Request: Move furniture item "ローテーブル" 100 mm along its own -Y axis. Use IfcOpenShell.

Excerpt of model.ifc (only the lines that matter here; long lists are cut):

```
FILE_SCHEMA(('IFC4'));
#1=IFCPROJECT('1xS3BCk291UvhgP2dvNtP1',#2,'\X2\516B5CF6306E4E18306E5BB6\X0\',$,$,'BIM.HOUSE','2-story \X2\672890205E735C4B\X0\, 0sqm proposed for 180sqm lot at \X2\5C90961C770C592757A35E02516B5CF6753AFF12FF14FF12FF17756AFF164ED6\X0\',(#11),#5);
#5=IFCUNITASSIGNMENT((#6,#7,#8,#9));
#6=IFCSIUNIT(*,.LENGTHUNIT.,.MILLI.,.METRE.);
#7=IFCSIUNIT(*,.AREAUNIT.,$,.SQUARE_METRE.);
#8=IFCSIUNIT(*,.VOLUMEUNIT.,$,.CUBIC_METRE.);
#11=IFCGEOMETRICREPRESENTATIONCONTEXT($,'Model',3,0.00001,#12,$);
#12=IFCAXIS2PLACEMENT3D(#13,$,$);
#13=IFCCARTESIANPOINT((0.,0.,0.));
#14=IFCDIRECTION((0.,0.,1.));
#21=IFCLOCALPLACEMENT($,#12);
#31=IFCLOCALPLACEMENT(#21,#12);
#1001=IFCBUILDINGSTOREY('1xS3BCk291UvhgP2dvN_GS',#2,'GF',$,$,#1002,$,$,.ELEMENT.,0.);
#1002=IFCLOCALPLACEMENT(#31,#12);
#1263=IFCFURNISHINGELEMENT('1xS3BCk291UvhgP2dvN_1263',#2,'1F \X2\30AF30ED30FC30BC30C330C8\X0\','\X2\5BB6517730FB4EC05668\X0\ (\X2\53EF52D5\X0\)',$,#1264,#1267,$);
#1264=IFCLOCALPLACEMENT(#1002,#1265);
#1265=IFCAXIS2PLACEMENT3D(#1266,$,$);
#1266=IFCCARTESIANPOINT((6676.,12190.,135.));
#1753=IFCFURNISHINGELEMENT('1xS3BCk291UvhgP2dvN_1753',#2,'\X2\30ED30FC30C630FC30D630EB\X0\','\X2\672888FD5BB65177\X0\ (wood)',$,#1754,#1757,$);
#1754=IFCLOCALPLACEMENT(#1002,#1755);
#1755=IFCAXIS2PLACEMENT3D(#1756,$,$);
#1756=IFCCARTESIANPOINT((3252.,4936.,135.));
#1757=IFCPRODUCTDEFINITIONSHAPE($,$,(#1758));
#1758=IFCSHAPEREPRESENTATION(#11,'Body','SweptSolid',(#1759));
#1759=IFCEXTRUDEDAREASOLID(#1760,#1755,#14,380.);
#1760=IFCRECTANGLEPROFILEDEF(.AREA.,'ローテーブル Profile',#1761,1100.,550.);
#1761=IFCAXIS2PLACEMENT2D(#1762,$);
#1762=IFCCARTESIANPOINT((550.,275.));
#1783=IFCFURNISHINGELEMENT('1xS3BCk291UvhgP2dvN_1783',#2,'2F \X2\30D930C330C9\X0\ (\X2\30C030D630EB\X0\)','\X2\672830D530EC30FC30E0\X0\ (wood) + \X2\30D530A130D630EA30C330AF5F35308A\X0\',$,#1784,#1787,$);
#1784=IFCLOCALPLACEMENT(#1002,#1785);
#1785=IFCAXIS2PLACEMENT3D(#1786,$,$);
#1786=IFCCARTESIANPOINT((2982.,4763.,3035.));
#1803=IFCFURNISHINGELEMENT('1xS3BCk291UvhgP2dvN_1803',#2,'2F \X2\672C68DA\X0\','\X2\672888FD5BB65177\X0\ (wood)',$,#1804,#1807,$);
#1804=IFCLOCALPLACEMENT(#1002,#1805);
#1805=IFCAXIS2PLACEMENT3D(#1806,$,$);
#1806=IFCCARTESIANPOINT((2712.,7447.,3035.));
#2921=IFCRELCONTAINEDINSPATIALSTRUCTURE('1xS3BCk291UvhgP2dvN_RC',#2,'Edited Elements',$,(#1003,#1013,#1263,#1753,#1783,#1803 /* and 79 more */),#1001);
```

```python
import ifcopenshell
import ifcopenshell.api.geometry
import ifcopenshell.util.placement
import ifcopenshell.util.unit

model = ifcopenshell.open("model.ifc")
unit_scale = ifcopenshell.util.unit.calculate_unit_scale(model)

item = model.by_guid("1xS3BCk291UvhgP2dvN_1753")
matrix = ifcopenshell.util.placement.get_local_placement(item.ObjectPlacement)
matrix[:3, 3] -= matrix[:3, 1] * 0.1 / unit_scale
ifcopenshell.api.geometry.edit_object_placement(model, product=item, matrix=matrix, is_si=False)

print(ifcopenshell.util.placement.get_local_placement(item.ObjectPlacement).round(3) + 0.0)

model.write("model_rev.ifc")
```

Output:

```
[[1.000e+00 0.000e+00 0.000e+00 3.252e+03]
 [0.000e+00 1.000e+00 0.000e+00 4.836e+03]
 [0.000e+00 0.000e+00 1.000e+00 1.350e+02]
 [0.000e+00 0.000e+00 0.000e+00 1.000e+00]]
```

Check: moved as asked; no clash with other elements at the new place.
